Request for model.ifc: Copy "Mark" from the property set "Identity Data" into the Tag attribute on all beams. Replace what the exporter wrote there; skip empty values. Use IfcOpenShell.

First a look at what the model holds.

```python
import ifcopenshell
import ifcopenshell.util.element

model = ifcopenshell.open("model.ifc")
print(model.schema)
beams = model.by_type("IfcBeam")
print(len(beams), "beams")
for e in beams[:8]:
    source = ifcopenshell.util.element.get_pset(e, "Identity Data", "Mark")
    target = e.Tag
    print(e.id(), repr(source), repr(target), sep=" | ")
```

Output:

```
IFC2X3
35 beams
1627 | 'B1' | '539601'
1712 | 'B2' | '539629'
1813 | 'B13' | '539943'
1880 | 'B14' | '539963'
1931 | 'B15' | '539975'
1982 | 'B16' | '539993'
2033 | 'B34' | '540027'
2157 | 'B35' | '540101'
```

```python
import ifcopenshell
import ifcopenshell.util.element

model = ifcopenshell.open("model.ifc")

count = 0
for e in model.by_type("IfcBeam"):
    value = ifcopenshell.util.element.get_pset(e, "Identity Data", "Mark")
    current = e.Tag
    if not value or not value.strip() or current == value:
        continue
    e.Tag = value
    count += 1

print(count, "beams updated")

model.write("model_updated.ifc")
```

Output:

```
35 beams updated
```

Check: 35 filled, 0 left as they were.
